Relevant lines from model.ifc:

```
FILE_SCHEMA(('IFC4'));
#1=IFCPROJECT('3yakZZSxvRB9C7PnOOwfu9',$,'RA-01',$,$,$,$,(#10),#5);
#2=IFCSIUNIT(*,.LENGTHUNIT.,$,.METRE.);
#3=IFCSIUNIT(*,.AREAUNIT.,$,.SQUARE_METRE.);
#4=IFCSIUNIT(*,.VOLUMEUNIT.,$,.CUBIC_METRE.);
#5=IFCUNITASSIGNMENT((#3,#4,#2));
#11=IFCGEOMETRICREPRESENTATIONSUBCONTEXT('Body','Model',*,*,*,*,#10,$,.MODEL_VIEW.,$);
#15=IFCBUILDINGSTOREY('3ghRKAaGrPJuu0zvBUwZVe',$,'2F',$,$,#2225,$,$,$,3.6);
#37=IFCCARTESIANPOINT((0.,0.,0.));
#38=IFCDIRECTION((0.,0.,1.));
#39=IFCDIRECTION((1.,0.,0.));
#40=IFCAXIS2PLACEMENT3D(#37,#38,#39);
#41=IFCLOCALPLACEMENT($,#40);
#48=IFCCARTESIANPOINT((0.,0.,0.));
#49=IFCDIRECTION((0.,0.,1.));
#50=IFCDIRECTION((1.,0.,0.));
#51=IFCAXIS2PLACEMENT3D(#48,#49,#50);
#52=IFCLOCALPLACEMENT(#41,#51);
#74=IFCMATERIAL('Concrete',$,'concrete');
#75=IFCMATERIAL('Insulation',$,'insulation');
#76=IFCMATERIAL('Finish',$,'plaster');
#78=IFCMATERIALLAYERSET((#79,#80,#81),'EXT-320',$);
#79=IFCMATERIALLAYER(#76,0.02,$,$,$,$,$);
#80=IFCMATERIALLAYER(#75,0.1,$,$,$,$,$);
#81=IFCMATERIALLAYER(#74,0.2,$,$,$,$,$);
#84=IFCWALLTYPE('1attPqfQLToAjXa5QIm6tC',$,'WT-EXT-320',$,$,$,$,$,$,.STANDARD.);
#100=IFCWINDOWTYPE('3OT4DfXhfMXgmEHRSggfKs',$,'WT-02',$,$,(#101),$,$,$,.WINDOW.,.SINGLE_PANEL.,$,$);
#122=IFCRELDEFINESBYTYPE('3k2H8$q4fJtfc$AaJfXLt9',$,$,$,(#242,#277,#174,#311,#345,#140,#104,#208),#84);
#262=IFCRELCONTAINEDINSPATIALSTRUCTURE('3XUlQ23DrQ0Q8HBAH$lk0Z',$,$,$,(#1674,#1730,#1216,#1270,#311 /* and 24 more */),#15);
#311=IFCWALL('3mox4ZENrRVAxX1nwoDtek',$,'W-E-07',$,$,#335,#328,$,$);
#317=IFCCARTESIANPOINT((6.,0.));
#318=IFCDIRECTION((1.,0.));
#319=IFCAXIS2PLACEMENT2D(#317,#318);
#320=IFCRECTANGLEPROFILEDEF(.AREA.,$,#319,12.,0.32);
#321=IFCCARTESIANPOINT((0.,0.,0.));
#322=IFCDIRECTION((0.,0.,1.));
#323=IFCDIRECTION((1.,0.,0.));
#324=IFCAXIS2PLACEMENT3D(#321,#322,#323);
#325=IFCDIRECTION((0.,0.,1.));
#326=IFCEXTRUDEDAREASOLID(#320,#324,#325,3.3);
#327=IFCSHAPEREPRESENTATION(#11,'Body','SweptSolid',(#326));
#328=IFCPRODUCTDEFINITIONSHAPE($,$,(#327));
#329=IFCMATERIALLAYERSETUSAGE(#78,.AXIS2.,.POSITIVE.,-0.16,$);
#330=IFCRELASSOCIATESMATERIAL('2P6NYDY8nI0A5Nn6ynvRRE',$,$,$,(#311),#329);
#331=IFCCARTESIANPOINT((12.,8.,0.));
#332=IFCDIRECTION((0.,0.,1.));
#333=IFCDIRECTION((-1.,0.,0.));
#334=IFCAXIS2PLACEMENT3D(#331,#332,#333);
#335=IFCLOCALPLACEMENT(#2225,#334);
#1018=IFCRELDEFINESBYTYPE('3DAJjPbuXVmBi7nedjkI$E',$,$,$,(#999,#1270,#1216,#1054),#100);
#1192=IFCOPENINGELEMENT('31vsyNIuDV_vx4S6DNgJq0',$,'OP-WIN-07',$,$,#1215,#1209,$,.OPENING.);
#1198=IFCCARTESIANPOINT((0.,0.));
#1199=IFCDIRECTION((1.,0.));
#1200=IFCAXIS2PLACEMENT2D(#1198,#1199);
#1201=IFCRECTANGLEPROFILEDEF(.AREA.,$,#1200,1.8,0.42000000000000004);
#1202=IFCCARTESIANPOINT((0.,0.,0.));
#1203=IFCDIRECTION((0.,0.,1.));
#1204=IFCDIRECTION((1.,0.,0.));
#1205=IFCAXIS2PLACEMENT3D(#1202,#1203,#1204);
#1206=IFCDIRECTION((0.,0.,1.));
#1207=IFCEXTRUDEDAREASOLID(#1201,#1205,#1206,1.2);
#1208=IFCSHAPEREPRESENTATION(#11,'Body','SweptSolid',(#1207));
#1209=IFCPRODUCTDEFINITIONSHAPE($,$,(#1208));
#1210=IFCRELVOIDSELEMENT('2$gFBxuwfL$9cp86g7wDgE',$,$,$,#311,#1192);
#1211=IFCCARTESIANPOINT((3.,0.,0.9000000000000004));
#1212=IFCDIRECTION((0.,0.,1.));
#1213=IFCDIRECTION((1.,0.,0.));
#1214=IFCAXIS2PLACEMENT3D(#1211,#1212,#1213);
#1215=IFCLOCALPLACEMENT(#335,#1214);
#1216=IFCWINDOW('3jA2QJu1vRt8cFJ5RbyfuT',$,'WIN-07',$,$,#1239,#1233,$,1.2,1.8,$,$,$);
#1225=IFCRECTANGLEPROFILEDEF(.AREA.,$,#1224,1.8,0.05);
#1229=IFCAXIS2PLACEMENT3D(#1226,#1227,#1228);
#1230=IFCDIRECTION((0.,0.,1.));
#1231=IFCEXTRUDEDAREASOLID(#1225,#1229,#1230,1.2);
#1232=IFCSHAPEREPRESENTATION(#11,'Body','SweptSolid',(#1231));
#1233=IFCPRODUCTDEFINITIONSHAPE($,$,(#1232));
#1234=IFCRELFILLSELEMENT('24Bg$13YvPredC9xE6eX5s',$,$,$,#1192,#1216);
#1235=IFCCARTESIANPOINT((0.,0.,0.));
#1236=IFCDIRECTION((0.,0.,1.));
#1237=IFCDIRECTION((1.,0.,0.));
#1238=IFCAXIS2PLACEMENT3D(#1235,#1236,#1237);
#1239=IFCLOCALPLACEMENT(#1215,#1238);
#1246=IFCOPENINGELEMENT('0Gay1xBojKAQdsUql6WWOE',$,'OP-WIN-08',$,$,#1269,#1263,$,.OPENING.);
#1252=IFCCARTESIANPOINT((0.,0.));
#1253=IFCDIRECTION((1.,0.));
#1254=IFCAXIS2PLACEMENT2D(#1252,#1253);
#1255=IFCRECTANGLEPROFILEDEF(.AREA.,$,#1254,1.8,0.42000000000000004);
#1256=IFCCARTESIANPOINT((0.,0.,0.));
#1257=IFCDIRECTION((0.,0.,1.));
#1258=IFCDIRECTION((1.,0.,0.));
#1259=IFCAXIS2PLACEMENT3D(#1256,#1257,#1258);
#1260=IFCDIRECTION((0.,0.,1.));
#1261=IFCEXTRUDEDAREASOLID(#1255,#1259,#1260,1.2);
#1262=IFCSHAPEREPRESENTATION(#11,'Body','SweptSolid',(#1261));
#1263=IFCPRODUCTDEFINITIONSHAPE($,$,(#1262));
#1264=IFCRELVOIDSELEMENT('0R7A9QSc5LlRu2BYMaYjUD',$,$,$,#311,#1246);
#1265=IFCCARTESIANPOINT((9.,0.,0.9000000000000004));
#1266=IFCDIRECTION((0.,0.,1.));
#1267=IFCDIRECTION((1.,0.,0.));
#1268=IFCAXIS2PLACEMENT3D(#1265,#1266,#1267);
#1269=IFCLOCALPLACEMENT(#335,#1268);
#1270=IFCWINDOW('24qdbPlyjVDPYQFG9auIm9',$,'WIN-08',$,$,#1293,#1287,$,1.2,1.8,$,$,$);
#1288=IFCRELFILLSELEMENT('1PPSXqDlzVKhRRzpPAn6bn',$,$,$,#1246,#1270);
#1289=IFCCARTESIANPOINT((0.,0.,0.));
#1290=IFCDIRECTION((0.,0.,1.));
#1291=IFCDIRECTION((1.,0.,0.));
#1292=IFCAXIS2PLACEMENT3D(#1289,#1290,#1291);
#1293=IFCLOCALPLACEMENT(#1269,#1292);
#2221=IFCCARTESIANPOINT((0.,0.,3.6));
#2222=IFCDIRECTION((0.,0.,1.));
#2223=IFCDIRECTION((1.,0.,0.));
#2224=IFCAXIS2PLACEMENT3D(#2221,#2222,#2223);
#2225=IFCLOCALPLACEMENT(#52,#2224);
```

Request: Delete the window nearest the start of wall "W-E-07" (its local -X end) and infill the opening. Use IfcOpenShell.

```python
import ifcopenshell
import ifcopenshell.api.feature
import ifcopenshell.api.root
import ifcopenshell.geom
import ifcopenshell.util.shape

model = ifcopenshell.open("model.ifc")
settings = ifcopenshell.geom.settings()


def volume(element):
    """Net volume in cubic metres, openings subtracted."""
    shape = ifcopenshell.geom.create_shape(settings, element)
    return ifcopenshell.util.shape.get_volume(shape.geometry)


window = model.by_id(1216)
opening = window.FillsVoids[0].RelatingOpeningElement
wall = opening.VoidsElements[0].RelatingBuildingElement
before = volume(wall)

ifcopenshell.api.root.remove_product(model, product=window)
ifcopenshell.api.feature.remove_feature(model, feature=opening)

after = volume(wall)

print(f"wall volume {before:.3f} -> {after:.3f} m3")

model.write("model_v2.ifc")
```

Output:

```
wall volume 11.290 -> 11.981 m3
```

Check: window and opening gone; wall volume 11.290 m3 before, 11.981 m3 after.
